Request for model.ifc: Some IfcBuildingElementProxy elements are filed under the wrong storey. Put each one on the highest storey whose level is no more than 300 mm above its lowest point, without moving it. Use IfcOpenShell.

First a look at what the model holds.

```python
import ifcopenshell
import ifcopenshell.util.element
import ifcopenshell.util.placement

model = ifcopenshell.open("model.ifc")
print(model.schema)
for storey in model.by_type("IfcBuildingStorey"):
    level = ifcopenshell.util.placement.get_storey_elevation(storey)
    count = sum(e.is_a("IfcBuildingElementProxy") for e in ifcopenshell.util.element.get_contained(storey))
    print(storey.id(), storey.Name, round(level, 3), count, sep=" | ")
```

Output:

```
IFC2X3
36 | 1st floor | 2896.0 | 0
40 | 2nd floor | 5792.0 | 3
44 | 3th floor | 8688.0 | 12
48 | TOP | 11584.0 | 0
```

```python
import ifcopenshell
import ifcopenshell.api.spatial
import ifcopenshell.geom
import ifcopenshell.util.element
import ifcopenshell.util.placement
import ifcopenshell.util.shape
import ifcopenshell.util.unit

model = ifcopenshell.open("model.ifc")
unit_scale = ifcopenshell.util.unit.calculate_unit_scale(model)
settings = ifcopenshell.geom.settings()

levels = sorted(
    ((ifcopenshell.util.placement.get_storey_elevation(s) * unit_scale, s) for s in model.by_type("IfcBuildingStorey")),
    key=lambda pair: pair[0],
)

for e in model.by_type("IfcBuildingElementProxy"):
    current = e.ContainedInStructure[0].RelatingStructure if e.ContainedInStructure else None
    if current is None or not current.is_a("IfcBuildingStorey"):
        continue
    shape = ifcopenshell.geom.create_shape(settings, e)
    bottom = ifcopenshell.util.shape.get_shape_bottom_elevation(shape, shape.geometry)
    below = [s for level, s in levels if level <= bottom + 0.3]
    storey = below[-1] if below else levels[0][1]
    if storey != current:
        # assign_container keeps the world position.
        ifcopenshell.api.spatial.assign_container(model, products=[e], relating_structure=storey)
        print(e.id(), current.Name, "->", storey.Name)

model.write("model-out.ifc")
```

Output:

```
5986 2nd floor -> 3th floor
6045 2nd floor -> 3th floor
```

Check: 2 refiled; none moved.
